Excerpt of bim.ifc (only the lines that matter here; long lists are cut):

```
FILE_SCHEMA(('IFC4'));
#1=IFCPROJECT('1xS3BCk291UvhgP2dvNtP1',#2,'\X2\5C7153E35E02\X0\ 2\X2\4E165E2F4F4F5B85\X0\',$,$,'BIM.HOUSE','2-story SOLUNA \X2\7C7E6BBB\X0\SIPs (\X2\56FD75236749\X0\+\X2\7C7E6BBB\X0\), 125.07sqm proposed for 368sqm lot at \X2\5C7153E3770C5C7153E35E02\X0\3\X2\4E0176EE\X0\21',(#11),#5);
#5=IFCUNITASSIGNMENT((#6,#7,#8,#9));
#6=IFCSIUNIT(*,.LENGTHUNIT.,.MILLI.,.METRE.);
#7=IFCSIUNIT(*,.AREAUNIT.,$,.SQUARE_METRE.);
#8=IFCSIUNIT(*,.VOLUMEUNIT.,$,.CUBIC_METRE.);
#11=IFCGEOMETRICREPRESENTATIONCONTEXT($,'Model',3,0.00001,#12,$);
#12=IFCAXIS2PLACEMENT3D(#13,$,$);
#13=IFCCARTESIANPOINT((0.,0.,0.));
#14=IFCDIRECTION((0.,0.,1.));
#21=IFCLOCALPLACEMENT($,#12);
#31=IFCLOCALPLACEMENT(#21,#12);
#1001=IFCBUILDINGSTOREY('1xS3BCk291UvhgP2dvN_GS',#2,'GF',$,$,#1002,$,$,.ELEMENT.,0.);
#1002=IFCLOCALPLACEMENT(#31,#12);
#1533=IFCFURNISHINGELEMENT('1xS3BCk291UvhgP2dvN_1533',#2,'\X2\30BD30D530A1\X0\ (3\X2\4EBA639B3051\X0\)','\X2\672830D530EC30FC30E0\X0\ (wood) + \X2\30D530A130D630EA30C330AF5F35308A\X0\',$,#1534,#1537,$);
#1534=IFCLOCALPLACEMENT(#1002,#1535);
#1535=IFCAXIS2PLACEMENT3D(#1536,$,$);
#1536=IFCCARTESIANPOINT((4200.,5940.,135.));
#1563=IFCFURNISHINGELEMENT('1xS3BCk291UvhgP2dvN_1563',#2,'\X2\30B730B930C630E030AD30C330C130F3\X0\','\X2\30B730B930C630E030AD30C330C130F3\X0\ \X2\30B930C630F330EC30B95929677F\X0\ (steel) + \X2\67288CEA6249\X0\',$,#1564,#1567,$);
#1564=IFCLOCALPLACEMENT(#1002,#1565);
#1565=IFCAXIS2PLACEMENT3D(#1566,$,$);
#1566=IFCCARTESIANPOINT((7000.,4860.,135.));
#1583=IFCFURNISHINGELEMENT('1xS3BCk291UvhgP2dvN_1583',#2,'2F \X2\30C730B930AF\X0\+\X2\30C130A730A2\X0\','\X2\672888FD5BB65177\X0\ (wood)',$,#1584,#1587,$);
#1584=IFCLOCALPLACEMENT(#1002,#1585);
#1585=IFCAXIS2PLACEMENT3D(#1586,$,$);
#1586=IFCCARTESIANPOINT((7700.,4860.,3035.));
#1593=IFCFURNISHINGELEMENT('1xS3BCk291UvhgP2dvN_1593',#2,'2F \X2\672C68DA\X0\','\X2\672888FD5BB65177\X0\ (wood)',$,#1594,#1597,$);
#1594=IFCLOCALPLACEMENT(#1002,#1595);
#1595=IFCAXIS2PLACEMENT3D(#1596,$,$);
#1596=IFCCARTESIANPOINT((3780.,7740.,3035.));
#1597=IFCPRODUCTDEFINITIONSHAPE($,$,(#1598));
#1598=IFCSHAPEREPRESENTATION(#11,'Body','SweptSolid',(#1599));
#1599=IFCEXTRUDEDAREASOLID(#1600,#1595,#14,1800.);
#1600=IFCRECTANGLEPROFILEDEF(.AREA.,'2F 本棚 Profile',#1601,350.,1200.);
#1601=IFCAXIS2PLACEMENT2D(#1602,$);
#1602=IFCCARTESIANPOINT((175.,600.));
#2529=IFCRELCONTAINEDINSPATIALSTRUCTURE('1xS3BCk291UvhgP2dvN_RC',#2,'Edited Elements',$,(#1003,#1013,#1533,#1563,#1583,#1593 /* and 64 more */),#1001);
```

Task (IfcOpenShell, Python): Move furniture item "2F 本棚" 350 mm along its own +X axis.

```python
import ifcopenshell
import ifcopenshell.api.geometry
import ifcopenshell.util.placement

model = ifcopenshell.open("bim.ifc")

item = model.by_id(1593)
matrix = ifcopenshell.util.placement.get_local_placement(item.ObjectPlacement)
matrix[:3, 3] += matrix[:3, 0] * 350.0
ifcopenshell.api.geometry.edit_object_placement(model, product=item, matrix=matrix, is_si=False)

print(ifcopenshell.util.placement.get_local_placement(item.ObjectPlacement).round(3) + 0.0)

model.write("bim_updated.ifc")
```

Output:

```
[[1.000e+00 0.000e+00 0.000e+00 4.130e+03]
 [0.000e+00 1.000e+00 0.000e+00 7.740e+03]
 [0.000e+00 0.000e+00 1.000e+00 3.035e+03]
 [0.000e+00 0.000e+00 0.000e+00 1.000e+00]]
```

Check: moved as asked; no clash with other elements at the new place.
